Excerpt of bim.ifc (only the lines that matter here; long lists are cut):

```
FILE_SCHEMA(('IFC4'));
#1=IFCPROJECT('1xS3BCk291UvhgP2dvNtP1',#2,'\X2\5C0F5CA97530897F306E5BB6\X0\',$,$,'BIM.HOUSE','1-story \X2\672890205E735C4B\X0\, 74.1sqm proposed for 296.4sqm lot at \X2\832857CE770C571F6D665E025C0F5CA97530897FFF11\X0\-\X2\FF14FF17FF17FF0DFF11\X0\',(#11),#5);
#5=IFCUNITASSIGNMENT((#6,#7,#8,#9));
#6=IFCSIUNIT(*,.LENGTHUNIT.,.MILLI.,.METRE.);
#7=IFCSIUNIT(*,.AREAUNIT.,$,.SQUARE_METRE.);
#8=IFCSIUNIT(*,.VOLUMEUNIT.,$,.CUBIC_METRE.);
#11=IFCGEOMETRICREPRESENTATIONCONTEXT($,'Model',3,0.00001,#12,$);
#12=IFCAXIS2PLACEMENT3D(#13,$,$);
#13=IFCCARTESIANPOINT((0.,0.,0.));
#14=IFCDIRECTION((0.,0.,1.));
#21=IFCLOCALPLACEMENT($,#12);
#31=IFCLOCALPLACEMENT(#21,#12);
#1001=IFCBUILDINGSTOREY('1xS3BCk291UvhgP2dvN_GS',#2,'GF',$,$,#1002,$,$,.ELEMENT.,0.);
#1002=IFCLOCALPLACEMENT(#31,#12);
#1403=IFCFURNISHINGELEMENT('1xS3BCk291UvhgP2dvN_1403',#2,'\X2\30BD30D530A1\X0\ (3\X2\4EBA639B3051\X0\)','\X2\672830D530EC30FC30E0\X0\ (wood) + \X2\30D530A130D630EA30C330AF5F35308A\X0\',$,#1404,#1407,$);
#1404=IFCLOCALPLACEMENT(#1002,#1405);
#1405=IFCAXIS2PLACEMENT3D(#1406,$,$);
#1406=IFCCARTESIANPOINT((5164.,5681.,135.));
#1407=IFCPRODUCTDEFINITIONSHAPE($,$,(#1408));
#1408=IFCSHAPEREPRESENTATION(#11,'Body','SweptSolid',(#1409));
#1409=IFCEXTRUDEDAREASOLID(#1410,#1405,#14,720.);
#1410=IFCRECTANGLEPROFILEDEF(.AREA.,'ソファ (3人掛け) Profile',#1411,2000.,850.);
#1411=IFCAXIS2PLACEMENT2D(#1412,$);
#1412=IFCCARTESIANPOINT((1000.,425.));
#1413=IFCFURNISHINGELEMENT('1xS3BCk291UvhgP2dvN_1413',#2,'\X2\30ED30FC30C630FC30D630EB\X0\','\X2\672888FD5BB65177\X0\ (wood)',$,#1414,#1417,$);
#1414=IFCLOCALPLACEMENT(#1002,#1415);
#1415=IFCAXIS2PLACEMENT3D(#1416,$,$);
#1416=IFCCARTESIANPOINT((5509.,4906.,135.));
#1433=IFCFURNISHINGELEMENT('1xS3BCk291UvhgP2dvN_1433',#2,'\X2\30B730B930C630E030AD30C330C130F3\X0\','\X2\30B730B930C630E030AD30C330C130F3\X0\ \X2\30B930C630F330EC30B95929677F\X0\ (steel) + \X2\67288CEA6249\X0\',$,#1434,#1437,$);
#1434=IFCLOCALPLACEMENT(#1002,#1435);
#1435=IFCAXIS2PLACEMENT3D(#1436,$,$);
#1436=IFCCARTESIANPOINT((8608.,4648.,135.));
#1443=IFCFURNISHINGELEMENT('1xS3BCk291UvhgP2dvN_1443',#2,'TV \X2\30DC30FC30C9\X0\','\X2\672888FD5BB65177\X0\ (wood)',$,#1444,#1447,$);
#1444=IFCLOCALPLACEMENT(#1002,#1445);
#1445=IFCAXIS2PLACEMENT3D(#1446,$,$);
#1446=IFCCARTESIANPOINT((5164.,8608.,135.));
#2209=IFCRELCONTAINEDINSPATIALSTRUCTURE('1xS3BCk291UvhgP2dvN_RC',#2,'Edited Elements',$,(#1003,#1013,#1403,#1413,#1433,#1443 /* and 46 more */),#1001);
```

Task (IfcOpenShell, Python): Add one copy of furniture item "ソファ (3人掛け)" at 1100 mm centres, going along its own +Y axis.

```python
import ifcopenshell
import ifcopenshell.api.geometry
import ifcopenshell.api.root
import ifcopenshell.util.element
import ifcopenshell.util.placement
import ifcopenshell.util.unit

model = ifcopenshell.open("bim.ifc")
unit_scale = ifcopenshell.util.unit.calculate_unit_scale(model)


def reuse_history(source, copy):
    """copy_class also copies each property set's owner history, people and application; keep the originals."""
    for rel in copy.IsDefinedBy:
        if rel.is_a("IfcRelDefinesByProperties") and (history := rel.RelatingPropertyDefinition.OwnerHistory):
            rel.RelatingPropertyDefinition.OwnerHistory = source.OwnerHistory
            ifcopenshell.util.element.remove_deep2(model, history)


source = model.by_guid("1xS3BCk291UvhgP2dvN_1403")
base = ifcopenshell.util.placement.get_local_placement(source.ObjectPlacement)
step = base[:3, 1] * 1.1 / unit_scale

for i in range(1, 2):
    copy = ifcopenshell.api.root.copy_class(model, product=source)
    copy.Representation = ifcopenshell.util.element.copy_deep(
        model, source.Representation, exclude=["IfcGeometricRepresentationContext", "IfcRepresentationMap"]
    )
    reuse_history(source, copy)
    matrix = base.copy()
    matrix[:3, 3] += i * step
    print("added at", matrix[:3, 3].round(3) + 0.0)
    ifcopenshell.api.geometry.edit_object_placement(model, product=copy, matrix=matrix, is_si=False)

model.write("bim_rev.ifc")
```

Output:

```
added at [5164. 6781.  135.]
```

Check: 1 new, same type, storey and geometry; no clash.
